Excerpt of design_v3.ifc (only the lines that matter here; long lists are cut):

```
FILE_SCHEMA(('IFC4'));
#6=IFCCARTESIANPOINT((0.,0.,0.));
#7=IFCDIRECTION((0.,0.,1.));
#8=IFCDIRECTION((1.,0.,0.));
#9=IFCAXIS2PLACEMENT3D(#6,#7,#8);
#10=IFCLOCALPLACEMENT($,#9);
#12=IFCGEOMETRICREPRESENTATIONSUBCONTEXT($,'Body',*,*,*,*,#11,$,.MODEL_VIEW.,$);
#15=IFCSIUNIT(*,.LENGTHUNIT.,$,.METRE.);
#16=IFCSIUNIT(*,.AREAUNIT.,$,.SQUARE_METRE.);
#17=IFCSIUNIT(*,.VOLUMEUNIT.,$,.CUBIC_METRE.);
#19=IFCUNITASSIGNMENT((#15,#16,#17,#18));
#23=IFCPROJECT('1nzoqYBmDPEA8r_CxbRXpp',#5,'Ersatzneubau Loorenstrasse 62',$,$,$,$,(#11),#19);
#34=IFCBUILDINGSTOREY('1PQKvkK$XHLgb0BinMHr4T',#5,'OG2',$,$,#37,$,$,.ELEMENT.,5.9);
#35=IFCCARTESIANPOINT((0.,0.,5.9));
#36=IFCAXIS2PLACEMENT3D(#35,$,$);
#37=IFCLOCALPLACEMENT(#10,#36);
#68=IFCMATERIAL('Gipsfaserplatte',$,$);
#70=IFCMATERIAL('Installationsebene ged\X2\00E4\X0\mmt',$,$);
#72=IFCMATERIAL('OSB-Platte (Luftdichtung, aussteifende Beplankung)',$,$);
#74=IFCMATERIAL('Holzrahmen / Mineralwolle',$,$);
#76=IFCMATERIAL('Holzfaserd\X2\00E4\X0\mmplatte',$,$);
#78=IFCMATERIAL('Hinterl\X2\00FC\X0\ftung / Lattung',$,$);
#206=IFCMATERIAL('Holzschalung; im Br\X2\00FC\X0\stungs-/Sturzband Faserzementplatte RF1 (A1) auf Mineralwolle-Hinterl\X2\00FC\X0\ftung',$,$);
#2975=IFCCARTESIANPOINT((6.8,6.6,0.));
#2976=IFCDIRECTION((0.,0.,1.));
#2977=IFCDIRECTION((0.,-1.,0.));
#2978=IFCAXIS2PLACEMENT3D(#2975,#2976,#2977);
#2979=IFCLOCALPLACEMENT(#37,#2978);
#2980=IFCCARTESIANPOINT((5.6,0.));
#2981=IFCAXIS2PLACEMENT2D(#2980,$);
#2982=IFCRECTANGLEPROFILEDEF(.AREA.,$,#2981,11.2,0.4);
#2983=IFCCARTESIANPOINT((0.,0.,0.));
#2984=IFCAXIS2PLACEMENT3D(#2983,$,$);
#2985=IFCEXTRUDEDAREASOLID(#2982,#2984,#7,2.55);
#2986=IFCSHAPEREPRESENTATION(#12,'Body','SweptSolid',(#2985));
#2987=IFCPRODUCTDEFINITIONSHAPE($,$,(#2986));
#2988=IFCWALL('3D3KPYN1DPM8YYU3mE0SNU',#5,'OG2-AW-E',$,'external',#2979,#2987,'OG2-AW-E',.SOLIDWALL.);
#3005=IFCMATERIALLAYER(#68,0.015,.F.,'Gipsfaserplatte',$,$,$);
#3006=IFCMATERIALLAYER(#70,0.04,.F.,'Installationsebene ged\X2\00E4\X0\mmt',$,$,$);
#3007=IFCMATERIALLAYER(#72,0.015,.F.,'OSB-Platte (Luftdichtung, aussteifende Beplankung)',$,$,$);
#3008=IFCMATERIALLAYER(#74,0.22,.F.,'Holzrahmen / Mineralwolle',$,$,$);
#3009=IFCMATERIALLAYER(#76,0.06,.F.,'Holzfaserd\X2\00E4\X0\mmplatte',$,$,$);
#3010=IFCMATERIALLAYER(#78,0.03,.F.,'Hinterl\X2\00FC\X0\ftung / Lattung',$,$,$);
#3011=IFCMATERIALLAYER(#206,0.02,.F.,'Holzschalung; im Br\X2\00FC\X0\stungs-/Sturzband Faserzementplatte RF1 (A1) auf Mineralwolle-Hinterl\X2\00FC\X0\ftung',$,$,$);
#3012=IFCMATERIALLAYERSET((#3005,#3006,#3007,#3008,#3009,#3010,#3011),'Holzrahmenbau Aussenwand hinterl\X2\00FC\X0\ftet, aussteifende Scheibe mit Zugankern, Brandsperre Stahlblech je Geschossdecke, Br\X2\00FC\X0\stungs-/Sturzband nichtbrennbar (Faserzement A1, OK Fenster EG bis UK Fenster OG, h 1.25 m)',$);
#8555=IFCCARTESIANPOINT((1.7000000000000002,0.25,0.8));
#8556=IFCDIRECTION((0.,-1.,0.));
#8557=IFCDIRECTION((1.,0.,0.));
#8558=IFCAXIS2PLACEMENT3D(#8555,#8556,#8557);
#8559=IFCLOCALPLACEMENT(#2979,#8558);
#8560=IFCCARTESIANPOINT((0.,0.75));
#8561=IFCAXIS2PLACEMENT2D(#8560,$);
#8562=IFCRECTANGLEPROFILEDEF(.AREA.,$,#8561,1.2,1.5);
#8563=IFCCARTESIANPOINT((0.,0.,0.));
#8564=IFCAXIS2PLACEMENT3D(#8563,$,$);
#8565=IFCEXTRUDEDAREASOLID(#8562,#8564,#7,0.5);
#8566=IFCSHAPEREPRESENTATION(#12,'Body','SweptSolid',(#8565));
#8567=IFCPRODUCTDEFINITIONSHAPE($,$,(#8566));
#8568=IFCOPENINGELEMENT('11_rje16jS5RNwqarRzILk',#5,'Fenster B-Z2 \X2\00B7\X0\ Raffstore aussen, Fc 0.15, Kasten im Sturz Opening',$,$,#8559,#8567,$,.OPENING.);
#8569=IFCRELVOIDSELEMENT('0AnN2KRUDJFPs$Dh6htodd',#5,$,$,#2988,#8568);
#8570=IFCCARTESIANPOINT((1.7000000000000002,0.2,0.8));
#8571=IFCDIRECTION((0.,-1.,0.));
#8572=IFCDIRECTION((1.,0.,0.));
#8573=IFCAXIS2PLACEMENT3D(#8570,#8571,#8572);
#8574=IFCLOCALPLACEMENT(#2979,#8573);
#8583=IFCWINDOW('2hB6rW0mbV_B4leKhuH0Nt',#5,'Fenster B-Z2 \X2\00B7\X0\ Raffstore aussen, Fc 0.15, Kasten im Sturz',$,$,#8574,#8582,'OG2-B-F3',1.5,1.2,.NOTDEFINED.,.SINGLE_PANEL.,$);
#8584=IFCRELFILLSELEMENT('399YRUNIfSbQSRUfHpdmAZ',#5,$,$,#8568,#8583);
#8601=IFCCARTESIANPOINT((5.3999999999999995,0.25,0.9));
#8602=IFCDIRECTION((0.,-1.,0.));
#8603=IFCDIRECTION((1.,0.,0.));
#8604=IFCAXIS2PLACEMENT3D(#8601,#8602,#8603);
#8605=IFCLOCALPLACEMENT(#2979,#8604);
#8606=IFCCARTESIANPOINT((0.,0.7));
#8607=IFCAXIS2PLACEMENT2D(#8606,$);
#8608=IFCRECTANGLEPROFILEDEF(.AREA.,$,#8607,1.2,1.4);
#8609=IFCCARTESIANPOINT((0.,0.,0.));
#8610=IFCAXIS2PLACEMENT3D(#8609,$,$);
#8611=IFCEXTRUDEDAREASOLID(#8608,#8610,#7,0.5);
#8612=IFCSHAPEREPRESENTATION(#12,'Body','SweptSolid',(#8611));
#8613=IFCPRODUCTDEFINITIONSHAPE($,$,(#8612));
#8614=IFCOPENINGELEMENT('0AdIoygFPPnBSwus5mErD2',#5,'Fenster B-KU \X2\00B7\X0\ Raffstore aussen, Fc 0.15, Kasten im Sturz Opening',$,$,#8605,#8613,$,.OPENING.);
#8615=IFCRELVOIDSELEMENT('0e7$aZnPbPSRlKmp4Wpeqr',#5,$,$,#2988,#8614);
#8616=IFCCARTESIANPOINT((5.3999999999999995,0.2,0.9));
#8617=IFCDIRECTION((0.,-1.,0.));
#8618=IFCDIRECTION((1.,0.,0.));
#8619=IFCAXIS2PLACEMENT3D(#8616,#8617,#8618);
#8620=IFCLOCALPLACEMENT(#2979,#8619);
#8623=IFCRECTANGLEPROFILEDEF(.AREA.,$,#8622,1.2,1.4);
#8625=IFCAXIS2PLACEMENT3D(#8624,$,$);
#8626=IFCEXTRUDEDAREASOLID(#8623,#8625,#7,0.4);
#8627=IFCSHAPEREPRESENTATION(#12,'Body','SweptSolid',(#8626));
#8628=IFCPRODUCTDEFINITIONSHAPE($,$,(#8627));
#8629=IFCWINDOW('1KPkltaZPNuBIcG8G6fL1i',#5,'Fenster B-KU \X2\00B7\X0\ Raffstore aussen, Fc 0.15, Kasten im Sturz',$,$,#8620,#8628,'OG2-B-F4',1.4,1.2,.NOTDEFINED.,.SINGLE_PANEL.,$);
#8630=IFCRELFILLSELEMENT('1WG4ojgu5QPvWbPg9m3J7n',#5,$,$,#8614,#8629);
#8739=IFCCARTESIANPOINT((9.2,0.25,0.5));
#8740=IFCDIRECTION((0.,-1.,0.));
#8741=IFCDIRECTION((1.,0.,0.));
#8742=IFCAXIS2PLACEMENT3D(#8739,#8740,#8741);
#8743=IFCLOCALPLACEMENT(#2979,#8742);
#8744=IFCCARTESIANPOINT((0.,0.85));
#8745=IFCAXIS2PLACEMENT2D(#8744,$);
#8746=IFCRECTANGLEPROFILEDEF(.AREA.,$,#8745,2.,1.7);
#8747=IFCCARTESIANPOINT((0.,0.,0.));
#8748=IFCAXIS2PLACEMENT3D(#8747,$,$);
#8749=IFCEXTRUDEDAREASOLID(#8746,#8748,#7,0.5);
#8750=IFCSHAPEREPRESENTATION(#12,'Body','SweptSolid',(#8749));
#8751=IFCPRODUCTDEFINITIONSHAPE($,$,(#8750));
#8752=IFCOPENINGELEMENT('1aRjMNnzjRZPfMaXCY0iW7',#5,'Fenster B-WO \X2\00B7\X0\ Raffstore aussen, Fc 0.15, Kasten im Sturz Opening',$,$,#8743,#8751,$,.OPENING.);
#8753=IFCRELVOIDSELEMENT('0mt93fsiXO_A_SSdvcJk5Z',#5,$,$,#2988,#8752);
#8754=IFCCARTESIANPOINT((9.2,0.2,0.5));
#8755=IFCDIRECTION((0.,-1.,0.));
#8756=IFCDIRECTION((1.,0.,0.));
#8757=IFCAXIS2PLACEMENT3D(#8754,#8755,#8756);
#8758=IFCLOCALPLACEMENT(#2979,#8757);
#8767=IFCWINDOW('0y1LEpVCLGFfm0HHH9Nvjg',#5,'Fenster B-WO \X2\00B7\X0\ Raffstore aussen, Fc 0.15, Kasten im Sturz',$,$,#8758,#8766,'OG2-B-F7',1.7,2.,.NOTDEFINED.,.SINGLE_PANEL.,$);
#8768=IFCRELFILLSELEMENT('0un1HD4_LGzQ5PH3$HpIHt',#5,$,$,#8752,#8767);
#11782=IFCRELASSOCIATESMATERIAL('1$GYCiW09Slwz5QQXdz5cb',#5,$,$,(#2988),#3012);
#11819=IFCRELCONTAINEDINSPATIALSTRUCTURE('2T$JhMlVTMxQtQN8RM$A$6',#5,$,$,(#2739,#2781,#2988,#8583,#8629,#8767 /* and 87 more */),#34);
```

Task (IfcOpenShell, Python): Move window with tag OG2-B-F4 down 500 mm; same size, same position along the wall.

```python
import numpy as np
import ifcopenshell
import ifcopenshell.api.geometry
import ifcopenshell.util.placement
import ifcopenshell.util.unit

model = ifcopenshell.open("design_v3.ifc")
unit_scale = ifcopenshell.util.unit.calculate_unit_scale(model)

window = model.by_guid("1KPkltaZPNuBIcG8G6fL1i")
opening = window.FillsVoids[0].RelatingOpeningElement
dz = -0.5 / unit_scale

shift = np.array([0.0, 0.0, dz])
# The window is not placed relative to its opening, so move both.
for product in (opening, window):
    matrix = ifcopenshell.util.placement.get_local_placement(product.ObjectPlacement)
    matrix[:3, 3] += shift
    ifcopenshell.api.geometry.edit_object_placement(model, product=product, matrix=matrix, is_si=False)

print(f"moved by {dz * unit_scale:+.3f} m")

model.write("design_v3_updated.ifc")
```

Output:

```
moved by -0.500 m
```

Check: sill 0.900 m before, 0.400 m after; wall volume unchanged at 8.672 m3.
